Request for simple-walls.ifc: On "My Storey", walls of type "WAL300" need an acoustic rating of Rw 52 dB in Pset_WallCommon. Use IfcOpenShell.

First a look at what the model holds.

```python
import ifcopenshell
import ifcopenshell.util.element

model = ifcopenshell.open("simple-walls.ifc")
print(model.schema)
storey = next(s for s in model.by_type("IfcBuildingStorey") if s.Name == "My Storey")
walls = [e for e in ifcopenshell.util.element.get_decomposition(storey) if e.is_a("IfcWall")]
seen = {}
for e in walls:
    element_type = ifcopenshell.util.element.get_type(e)
    key = (element_type.Name if element_type != e and element_type else None, ifcopenshell.util.element.get_pset(e, "Pset_WallCommon", "AcousticRating"))
    seen[key] = seen.get(key, 0) + 1
for (name, value), count in sorted(seen.items(), key=str):
    print(count, "x", name, "|", value)
```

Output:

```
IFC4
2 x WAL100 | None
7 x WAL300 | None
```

```python
import ifcopenshell
import ifcopenshell.api.pset
import ifcopenshell.util.element

model = ifcopenshell.open("simple-walls.ifc")

storey = next(s for s in model.by_type("IfcBuildingStorey") if s.Name == "My Storey")
walls = [e for e in ifcopenshell.util.element.get_decomposition(storey) if e.is_a("IfcWall")]

count = 0
for e in walls:
    element_type = ifcopenshell.util.element.get_type(e)
    if element_type in (None, e) or element_type.Name != "WAL300":
        continue
    # add_pset returns the element's existing set when there is one.
    pset = ifcopenshell.api.pset.add_pset(model, product=e, name="Pset_WallCommon")
    ifcopenshell.api.pset.edit_pset(model, pset=pset, properties={"AcousticRating": "Rw 52 dB"})
    count += 1

print(count, "walls updated")

model.write("simple-walls_edited.ifc")
```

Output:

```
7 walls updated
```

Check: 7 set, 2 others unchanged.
